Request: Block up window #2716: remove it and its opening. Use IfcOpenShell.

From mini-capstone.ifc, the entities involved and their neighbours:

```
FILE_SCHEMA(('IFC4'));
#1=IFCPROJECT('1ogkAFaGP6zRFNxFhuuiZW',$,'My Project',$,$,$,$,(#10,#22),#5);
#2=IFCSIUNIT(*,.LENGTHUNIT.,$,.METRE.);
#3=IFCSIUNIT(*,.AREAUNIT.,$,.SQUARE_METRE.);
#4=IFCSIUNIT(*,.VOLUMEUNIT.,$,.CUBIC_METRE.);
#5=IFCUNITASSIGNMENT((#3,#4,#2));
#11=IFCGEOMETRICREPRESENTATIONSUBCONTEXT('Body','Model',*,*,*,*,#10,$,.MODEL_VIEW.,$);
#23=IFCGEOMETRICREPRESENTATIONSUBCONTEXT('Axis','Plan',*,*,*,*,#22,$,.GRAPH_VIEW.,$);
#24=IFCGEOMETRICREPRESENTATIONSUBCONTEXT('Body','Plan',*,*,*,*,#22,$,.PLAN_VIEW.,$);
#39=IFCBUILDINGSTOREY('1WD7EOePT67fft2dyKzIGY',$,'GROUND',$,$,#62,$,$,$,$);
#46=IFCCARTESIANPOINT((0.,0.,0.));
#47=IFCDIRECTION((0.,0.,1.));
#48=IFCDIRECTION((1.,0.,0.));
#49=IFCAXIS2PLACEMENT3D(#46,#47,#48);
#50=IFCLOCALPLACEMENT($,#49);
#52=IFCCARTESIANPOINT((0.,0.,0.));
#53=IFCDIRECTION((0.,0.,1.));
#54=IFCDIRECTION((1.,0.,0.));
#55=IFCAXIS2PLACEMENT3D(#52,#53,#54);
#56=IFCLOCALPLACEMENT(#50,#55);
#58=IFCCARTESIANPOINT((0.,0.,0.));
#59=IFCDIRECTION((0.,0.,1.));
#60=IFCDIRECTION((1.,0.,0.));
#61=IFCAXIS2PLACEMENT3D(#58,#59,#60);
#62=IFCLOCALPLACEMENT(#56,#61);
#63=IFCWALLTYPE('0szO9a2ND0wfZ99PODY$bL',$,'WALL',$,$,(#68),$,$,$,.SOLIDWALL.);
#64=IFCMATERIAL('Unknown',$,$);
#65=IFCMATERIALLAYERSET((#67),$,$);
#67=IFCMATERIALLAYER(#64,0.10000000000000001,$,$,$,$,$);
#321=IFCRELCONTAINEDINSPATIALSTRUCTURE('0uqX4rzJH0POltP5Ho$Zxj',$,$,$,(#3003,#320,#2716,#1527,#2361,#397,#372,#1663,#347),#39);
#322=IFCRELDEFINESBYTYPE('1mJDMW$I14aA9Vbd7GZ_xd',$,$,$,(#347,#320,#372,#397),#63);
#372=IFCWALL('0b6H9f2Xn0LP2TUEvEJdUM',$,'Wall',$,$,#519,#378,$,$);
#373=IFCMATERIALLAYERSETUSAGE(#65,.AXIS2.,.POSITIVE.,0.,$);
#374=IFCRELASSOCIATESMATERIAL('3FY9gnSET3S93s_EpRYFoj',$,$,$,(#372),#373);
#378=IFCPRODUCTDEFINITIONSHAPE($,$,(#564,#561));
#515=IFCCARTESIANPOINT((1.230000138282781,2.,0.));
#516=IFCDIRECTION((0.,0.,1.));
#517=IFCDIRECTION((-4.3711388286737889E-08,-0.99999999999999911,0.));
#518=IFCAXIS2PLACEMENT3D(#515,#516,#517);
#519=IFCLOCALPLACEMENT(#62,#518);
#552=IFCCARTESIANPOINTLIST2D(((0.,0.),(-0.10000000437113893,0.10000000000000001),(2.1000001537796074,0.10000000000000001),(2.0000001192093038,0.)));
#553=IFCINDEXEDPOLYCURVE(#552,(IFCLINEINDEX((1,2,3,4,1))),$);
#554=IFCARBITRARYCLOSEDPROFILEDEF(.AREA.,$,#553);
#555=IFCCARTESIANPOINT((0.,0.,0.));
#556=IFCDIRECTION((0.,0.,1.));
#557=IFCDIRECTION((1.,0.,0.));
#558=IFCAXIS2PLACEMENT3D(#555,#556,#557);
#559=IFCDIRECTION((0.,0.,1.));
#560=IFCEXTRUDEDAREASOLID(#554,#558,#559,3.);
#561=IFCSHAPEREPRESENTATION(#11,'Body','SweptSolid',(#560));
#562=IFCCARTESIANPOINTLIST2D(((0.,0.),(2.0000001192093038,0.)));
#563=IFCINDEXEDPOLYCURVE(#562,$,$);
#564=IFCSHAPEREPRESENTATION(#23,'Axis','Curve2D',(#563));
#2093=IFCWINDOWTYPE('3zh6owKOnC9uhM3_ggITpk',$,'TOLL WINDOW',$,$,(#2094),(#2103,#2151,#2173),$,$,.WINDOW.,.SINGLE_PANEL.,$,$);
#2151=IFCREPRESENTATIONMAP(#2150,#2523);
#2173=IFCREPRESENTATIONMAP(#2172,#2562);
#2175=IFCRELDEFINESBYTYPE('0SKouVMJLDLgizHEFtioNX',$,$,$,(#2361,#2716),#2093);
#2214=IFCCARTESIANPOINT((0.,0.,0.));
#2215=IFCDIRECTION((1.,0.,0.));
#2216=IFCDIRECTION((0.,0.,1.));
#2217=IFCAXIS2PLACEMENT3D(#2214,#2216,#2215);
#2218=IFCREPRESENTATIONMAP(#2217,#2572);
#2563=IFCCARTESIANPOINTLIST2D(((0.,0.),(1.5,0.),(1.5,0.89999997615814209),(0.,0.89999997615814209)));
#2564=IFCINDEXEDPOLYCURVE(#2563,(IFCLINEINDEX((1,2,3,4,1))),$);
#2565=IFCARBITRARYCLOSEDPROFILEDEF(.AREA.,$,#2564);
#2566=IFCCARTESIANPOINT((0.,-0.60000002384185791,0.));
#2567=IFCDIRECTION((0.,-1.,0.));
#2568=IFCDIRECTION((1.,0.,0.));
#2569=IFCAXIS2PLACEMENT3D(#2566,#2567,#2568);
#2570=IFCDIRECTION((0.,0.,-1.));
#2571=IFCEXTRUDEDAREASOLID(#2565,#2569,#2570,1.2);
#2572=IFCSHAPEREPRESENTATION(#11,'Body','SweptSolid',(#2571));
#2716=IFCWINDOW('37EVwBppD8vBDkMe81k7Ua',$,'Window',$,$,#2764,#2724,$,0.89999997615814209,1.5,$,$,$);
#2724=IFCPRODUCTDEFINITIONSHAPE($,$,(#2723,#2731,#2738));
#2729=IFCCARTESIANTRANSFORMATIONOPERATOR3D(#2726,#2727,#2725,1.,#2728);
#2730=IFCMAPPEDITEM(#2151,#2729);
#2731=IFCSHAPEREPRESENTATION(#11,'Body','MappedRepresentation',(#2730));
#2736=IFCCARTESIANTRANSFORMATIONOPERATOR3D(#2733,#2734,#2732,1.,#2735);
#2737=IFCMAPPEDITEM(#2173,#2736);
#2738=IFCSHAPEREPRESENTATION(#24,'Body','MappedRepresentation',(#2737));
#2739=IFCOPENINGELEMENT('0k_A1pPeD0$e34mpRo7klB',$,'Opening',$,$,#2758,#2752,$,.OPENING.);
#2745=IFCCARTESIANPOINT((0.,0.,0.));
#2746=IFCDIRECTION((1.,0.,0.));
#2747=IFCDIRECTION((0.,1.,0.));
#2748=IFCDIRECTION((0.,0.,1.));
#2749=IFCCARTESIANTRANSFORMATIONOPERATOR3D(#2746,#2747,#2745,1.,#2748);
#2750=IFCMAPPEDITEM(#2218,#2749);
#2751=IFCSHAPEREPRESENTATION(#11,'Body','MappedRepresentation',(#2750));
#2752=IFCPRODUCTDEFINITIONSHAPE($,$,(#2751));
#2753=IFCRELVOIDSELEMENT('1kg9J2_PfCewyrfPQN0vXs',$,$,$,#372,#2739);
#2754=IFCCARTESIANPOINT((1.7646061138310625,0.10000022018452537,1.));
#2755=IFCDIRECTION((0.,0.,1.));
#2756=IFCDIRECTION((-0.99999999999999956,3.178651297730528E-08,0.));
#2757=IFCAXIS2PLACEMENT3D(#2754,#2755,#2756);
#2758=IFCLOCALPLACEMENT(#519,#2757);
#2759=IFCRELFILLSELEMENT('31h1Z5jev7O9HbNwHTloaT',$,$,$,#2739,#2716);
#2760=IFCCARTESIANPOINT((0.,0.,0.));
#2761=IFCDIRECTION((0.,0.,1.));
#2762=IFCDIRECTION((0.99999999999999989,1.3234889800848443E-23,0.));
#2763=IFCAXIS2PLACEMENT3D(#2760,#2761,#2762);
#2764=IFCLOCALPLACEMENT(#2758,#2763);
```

```python
import ifcopenshell
import ifcopenshell.api.feature
import ifcopenshell.api.root
import ifcopenshell.geom
import ifcopenshell.util.shape

model = ifcopenshell.open("mini-capstone.ifc")
settings = ifcopenshell.geom.settings()


def volume(element):
    """Net volume in cubic metres, openings subtracted."""
    shape = ifcopenshell.geom.create_shape(settings, element)
    return ifcopenshell.util.shape.get_volume(shape.geometry)


window = model.by_id(2716)
opening = window.FillsVoids[0].RelatingOpeningElement
wall = opening.VoidsElements[0].RelatingBuildingElement
before = volume(wall)

ifcopenshell.api.root.remove_product(model, product=window)
ifcopenshell.api.feature.remove_feature(model, feature=opening)

after = volume(wall)

print(f"wall volume {before:.3f} -> {after:.3f} m3")

model.write("mini-capstone_rev.ifc")
```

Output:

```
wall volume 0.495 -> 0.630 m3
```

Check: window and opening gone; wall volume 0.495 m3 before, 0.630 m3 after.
